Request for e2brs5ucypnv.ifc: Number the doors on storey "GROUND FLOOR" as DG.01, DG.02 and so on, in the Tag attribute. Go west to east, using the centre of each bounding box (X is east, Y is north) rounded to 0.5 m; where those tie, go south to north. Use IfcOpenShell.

First a look at what the model holds.

```python
import ifcopenshell
import ifcopenshell.util.element
import ifcopenshell.util.placement

model = ifcopenshell.open("e2brs5ucypnv.ifc")
print(model.schema)
storey = next(s for s in model.by_type("IfcBuildingStorey") if s.Name == "GROUND FLOOR")
doors = [e for e in ifcopenshell.util.element.get_decomposition(storey) if e.is_a("IfcDoor")]
for e in sorted(doors, key=lambda e: e.id()):
    origin = ifcopenshell.util.placement.get_local_placement(e.ObjectPlacement)[:3, 3]
    print(e.id(), e.Tag, e.Name, origin.round(2) + 0.0, sep=" | ")
```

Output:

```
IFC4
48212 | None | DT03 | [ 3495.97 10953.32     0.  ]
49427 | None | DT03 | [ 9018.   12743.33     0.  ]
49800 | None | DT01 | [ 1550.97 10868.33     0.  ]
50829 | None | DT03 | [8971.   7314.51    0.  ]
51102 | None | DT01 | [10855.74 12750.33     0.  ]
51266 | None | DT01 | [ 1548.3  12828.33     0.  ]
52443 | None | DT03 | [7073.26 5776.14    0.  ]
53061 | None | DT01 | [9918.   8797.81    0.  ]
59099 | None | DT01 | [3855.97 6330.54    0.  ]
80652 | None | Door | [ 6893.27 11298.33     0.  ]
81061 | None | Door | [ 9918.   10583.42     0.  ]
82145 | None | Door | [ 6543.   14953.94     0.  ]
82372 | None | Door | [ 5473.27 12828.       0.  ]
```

```python
import ifcopenshell
import ifcopenshell.geom
import ifcopenshell.util.element
import ifcopenshell.util.shape

model = ifcopenshell.open("e2brs5ucypnv.ifc")
settings = ifcopenshell.geom.settings()
settings.set("use-world-coords", True)


def centre(element):
    shape = ifcopenshell.geom.create_shape(settings, element)
    return ifcopenshell.util.shape.get_bbox_centroid(shape.geometry)


storey = next(s for s in model.by_type("IfcBuildingStorey") if s.Name == "GROUND FLOOR")
doors = [e for e in ifcopenshell.util.element.get_decomposition(storey) if e.is_a("IfcDoor")]

# Insertion points can sit at a corner or the storey origin, so sort by the geometry (in metres).
centres = {e: centre(e) for e in doors}
doors.sort(key=lambda e: (round(centres[e][0] / 0.5), centres[e][1]))

for i, e in enumerate(doors, start=1):
    number = f"DG.{i:02d}"
    e.Tag = number
    print(e.id(), number)

model.write("e2brs5ucypnv_edited.ifc")
```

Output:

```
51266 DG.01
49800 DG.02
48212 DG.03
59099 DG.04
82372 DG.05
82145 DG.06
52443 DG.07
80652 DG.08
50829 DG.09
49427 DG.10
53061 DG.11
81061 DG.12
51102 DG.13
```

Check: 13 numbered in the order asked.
